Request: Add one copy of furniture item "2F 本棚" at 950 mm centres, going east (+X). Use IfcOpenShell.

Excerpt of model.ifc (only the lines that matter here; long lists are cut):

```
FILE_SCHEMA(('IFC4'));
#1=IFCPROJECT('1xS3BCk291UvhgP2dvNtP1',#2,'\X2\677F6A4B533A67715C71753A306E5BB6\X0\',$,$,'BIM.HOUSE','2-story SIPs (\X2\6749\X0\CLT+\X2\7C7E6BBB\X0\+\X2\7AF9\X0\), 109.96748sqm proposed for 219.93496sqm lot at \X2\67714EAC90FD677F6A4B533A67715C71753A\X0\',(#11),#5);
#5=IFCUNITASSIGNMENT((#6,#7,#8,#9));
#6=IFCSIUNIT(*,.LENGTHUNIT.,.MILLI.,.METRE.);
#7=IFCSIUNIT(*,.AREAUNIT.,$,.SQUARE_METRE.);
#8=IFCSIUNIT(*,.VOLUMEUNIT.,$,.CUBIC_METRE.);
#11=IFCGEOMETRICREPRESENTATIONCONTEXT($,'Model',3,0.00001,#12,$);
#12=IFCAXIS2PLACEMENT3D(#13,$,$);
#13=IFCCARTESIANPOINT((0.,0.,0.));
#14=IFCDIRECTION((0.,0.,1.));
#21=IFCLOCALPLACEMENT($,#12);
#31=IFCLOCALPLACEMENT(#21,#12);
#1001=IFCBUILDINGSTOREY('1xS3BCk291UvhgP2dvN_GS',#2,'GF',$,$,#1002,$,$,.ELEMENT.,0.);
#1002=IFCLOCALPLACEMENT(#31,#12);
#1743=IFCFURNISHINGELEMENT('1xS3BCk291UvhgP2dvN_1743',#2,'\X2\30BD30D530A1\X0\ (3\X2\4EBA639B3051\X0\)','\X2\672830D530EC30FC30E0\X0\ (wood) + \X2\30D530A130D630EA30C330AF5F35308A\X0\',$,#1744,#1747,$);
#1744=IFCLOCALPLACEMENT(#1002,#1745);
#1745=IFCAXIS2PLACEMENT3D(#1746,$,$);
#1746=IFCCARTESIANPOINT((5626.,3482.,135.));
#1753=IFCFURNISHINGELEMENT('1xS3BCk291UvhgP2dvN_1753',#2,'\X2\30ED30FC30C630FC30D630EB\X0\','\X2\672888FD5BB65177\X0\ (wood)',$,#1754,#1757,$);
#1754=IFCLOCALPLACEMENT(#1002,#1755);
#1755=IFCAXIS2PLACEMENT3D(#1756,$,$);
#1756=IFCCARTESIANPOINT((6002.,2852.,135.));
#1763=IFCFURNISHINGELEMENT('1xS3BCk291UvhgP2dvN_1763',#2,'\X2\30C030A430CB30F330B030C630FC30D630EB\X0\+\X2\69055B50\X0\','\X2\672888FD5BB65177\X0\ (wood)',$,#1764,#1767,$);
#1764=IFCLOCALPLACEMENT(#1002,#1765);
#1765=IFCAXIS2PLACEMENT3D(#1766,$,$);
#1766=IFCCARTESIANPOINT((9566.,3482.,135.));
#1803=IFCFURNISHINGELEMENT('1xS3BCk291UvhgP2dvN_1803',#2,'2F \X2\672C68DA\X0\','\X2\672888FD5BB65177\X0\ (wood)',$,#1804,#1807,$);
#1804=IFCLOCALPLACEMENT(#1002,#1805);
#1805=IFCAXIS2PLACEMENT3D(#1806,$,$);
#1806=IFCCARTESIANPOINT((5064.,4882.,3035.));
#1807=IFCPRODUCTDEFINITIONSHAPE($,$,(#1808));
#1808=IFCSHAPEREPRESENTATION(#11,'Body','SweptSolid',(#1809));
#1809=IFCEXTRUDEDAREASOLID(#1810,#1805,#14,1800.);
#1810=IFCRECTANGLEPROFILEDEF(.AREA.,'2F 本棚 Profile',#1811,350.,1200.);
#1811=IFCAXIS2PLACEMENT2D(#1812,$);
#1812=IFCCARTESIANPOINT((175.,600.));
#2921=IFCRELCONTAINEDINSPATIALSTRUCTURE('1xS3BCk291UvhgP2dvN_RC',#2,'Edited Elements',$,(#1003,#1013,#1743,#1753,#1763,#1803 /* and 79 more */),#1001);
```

```python
import numpy as np
import ifcopenshell
import ifcopenshell.api.geometry
import ifcopenshell.api.root
import ifcopenshell.util.element
import ifcopenshell.util.placement
import ifcopenshell.util.unit

model = ifcopenshell.open("model.ifc")
unit_scale = ifcopenshell.util.unit.calculate_unit_scale(model)


def reuse_history(source, copy):
    """copy_class also copies each property set's owner history, people and application; keep the originals."""
    for rel in copy.IsDefinedBy:
        if rel.is_a("IfcRelDefinesByProperties") and (history := rel.RelatingPropertyDefinition.OwnerHistory):
            rel.RelatingPropertyDefinition.OwnerHistory = source.OwnerHistory
            ifcopenshell.util.element.remove_deep2(model, history)


source = model.by_guid("1xS3BCk291UvhgP2dvN_1803")
base = ifcopenshell.util.placement.get_local_placement(source.ObjectPlacement)
step = np.array([1.0, 0.0, 0.0]) * 0.95 / unit_scale

for i in range(1, 2):
    copy = ifcopenshell.api.root.copy_class(model, product=source)
    copy.Representation = ifcopenshell.util.element.copy_deep(
        model, source.Representation, exclude=["IfcGeometricRepresentationContext", "IfcRepresentationMap"]
    )
    reuse_history(source, copy)
    matrix = base.copy()
    matrix[:3, 3] += i * step
    print("added at", matrix[:3, 3].round(3) + 0.0)
    ifcopenshell.api.geometry.edit_object_placement(model, product=copy, matrix=matrix, is_si=False)

model.write("model_edited.ifc")
```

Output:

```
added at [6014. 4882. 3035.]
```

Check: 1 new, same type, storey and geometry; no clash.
